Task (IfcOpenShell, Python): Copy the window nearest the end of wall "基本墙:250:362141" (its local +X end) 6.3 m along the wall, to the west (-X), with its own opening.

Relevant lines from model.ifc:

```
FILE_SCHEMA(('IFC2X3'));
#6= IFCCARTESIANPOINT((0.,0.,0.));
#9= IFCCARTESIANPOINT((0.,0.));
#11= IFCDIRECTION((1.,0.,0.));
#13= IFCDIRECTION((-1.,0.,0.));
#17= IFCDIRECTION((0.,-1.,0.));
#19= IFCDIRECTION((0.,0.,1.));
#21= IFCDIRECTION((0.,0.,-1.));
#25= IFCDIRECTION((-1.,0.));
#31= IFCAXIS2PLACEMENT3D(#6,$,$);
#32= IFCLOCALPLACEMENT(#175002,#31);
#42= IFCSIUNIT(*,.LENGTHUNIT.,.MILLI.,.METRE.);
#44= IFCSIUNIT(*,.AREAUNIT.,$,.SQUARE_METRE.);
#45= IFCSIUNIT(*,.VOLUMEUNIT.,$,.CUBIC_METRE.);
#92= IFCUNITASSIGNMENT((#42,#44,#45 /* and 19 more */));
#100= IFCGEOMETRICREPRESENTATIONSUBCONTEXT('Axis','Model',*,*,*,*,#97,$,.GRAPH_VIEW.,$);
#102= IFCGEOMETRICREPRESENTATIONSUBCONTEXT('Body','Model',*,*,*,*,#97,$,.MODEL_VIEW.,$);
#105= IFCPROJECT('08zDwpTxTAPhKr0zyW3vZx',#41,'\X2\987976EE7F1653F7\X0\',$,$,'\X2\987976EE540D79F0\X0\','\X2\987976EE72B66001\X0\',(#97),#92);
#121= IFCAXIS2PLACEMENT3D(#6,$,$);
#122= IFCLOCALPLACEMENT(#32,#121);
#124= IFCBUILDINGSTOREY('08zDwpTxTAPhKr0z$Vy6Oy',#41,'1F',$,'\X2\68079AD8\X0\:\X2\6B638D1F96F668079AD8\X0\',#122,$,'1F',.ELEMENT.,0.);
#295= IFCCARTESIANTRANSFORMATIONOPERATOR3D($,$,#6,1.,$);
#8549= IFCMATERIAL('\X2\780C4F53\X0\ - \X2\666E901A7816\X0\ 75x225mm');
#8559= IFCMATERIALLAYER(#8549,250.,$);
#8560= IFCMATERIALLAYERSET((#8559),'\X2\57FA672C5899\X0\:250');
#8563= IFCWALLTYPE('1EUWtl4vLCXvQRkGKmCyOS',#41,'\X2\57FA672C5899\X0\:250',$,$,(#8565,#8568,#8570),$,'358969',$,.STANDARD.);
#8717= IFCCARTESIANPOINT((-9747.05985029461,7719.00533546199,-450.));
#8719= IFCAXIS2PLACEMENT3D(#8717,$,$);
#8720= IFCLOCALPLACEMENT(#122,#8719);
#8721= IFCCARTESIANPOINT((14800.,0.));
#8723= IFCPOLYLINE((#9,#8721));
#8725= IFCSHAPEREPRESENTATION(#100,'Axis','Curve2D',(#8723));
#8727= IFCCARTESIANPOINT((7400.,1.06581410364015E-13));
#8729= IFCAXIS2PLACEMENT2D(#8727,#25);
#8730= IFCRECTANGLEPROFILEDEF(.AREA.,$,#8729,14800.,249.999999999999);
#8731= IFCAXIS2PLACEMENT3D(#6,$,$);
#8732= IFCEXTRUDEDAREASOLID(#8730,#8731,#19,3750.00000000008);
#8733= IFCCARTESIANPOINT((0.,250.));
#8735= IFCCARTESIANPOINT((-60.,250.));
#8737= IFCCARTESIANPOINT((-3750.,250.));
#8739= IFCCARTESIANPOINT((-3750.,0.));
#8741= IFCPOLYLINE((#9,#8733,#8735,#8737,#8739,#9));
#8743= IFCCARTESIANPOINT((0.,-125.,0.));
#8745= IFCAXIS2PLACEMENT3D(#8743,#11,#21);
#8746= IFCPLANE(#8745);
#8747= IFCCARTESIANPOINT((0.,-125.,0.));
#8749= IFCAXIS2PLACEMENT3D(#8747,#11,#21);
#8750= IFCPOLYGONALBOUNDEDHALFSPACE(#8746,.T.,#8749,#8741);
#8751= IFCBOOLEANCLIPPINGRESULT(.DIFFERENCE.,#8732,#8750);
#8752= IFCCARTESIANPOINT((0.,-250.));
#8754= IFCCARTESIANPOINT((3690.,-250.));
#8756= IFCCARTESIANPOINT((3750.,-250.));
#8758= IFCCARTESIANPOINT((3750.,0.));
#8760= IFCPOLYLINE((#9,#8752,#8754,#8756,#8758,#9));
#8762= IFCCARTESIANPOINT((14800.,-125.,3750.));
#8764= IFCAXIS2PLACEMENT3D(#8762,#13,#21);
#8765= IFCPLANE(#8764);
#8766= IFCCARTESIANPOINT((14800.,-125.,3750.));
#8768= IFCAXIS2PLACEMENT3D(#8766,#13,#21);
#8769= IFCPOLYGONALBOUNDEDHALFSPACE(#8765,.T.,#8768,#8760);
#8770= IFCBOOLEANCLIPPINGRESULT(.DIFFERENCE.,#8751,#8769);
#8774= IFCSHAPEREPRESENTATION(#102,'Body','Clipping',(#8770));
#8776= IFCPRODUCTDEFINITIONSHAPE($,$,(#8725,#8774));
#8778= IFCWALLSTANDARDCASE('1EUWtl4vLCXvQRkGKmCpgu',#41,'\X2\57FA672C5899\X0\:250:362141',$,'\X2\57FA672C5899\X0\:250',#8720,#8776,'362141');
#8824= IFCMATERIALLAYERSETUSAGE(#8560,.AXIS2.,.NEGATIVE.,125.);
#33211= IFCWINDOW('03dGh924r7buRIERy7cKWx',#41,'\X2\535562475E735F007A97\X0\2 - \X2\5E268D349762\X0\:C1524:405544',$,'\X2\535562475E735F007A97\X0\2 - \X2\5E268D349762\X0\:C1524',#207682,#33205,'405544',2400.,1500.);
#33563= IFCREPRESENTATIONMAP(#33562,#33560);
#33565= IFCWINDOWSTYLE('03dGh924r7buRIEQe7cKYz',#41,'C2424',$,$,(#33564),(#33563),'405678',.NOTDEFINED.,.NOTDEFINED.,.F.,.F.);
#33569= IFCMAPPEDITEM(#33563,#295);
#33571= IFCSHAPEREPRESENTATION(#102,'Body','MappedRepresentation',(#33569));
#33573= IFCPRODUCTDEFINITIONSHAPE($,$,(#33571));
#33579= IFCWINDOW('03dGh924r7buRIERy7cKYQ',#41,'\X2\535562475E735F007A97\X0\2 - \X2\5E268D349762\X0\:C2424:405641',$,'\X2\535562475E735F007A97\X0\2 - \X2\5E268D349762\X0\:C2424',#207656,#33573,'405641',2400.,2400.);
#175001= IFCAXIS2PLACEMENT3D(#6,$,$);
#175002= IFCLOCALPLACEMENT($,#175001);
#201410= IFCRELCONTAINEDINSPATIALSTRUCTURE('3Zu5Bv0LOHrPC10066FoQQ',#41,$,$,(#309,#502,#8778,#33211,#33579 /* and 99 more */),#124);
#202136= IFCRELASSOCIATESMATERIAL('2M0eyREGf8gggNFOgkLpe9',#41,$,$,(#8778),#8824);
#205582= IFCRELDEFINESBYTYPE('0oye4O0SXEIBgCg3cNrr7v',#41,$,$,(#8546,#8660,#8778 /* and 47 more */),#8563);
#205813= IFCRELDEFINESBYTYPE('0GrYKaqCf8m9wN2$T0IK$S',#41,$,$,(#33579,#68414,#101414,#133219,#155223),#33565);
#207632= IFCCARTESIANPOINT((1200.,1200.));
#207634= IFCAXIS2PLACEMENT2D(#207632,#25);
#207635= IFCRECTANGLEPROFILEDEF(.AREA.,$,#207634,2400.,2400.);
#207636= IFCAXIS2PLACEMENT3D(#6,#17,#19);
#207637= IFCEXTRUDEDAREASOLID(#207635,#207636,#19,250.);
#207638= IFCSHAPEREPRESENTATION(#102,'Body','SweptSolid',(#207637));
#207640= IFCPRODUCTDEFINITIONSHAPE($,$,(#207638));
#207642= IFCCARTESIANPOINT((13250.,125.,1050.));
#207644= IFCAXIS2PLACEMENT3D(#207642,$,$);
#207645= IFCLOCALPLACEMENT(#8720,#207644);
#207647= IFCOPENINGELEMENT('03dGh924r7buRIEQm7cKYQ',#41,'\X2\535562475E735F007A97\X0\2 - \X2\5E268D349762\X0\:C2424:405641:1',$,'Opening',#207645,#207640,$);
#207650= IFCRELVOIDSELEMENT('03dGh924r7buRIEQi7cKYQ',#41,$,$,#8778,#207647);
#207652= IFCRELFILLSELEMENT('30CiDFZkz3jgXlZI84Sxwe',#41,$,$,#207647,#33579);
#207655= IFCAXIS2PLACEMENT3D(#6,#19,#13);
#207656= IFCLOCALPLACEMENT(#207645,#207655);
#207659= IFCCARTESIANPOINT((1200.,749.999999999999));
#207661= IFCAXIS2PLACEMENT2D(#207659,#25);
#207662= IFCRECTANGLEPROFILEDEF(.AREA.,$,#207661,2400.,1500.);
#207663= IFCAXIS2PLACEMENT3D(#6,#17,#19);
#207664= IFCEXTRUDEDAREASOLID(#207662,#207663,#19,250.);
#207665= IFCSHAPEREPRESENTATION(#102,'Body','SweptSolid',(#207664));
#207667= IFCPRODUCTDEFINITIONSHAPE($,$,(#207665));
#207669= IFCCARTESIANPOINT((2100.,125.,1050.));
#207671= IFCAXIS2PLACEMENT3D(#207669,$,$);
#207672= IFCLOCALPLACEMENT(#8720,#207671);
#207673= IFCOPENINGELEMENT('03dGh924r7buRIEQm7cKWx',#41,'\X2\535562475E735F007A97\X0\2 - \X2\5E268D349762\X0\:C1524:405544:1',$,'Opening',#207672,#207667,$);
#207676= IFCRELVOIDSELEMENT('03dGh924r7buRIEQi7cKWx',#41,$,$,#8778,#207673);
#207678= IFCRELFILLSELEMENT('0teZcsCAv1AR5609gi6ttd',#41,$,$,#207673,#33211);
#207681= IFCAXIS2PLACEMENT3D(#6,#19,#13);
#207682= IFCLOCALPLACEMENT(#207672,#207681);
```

```python
import ifcopenshell
import ifcopenshell.api.feature
import ifcopenshell.api.geometry
import ifcopenshell.api.root
import ifcopenshell.geom
import ifcopenshell.util.element
import ifcopenshell.util.placement
import ifcopenshell.util.shape

model = ifcopenshell.open("model.ifc")
settings = ifcopenshell.geom.settings()


def volume(element):
    """Net volume in cubic metres, openings subtracted."""
    shape = ifcopenshell.geom.create_shape(settings, element)
    return ifcopenshell.util.shape.get_volume(shape.geometry)


def reuse_history(source, copy):
    """copy_class also copies each property set's owner history, people and application; keep the originals."""
    for rel in copy.IsDefinedBy:
        if rel.is_a("IfcRelDefinesByProperties") and (history := rel.RelatingPropertyDefinition.OwnerHistory):
            rel.RelatingPropertyDefinition.OwnerHistory = source.OwnerHistory
            ifcopenshell.util.element.remove_deep2(model, history)


window = model.by_guid("03dGh924r7buRIERy7cKYQ")
opening = window.FillsVoids[0].RelatingOpeningElement
wall = opening.VoidsElements[0].RelatingBuildingElement
before = volume(wall)
shift = ifcopenshell.util.placement.get_local_placement(wall.ObjectPlacement)[:3, 0] * -6300.0

# copy_class copies the void relationship, type, container and properties, but no geometry.
new_opening = ifcopenshell.api.root.copy_class(model, product=opening)
new_opening.Representation = ifcopenshell.util.element.copy_deep(
    model, opening.Representation, exclude=["IfcGeometricRepresentationContext", "IfcRepresentationMap"]
)
new_opening.Name = "单扇平开窗2 - 带贴面:C2424"
new_window = ifcopenshell.api.root.copy_class(model, product=window)
new_window.Representation = ifcopenshell.util.element.copy_deep(
    model, window.Representation, exclude=["IfcGeometricRepresentationContext", "IfcRepresentationMap"]
)
new_window.Name = "单扇平开窗2 - 带贴面:C2424"
new_window.Tag = None
reuse_history(window, new_window)
fills = ifcopenshell.api.feature.add_filling(model, opening=new_opening, element=new_window)
fills.OwnerHistory = new_window.OwnerHistory  # required in IFC2X3

for old, new in ((opening, new_opening), (window, new_window)):
    matrix = ifcopenshell.util.placement.get_local_placement(old.ObjectPlacement)
    matrix[:3, 3] += shift
    ifcopenshell.api.geometry.edit_object_placement(model, product=new, matrix=matrix, is_si=False)

after = volume(wall)

print(f"wall volume {before:.3f} -> {after:.3f} m3")

model.write("model_edited.ifc")
```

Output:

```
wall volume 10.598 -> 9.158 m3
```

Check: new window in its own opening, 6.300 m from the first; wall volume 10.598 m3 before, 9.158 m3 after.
